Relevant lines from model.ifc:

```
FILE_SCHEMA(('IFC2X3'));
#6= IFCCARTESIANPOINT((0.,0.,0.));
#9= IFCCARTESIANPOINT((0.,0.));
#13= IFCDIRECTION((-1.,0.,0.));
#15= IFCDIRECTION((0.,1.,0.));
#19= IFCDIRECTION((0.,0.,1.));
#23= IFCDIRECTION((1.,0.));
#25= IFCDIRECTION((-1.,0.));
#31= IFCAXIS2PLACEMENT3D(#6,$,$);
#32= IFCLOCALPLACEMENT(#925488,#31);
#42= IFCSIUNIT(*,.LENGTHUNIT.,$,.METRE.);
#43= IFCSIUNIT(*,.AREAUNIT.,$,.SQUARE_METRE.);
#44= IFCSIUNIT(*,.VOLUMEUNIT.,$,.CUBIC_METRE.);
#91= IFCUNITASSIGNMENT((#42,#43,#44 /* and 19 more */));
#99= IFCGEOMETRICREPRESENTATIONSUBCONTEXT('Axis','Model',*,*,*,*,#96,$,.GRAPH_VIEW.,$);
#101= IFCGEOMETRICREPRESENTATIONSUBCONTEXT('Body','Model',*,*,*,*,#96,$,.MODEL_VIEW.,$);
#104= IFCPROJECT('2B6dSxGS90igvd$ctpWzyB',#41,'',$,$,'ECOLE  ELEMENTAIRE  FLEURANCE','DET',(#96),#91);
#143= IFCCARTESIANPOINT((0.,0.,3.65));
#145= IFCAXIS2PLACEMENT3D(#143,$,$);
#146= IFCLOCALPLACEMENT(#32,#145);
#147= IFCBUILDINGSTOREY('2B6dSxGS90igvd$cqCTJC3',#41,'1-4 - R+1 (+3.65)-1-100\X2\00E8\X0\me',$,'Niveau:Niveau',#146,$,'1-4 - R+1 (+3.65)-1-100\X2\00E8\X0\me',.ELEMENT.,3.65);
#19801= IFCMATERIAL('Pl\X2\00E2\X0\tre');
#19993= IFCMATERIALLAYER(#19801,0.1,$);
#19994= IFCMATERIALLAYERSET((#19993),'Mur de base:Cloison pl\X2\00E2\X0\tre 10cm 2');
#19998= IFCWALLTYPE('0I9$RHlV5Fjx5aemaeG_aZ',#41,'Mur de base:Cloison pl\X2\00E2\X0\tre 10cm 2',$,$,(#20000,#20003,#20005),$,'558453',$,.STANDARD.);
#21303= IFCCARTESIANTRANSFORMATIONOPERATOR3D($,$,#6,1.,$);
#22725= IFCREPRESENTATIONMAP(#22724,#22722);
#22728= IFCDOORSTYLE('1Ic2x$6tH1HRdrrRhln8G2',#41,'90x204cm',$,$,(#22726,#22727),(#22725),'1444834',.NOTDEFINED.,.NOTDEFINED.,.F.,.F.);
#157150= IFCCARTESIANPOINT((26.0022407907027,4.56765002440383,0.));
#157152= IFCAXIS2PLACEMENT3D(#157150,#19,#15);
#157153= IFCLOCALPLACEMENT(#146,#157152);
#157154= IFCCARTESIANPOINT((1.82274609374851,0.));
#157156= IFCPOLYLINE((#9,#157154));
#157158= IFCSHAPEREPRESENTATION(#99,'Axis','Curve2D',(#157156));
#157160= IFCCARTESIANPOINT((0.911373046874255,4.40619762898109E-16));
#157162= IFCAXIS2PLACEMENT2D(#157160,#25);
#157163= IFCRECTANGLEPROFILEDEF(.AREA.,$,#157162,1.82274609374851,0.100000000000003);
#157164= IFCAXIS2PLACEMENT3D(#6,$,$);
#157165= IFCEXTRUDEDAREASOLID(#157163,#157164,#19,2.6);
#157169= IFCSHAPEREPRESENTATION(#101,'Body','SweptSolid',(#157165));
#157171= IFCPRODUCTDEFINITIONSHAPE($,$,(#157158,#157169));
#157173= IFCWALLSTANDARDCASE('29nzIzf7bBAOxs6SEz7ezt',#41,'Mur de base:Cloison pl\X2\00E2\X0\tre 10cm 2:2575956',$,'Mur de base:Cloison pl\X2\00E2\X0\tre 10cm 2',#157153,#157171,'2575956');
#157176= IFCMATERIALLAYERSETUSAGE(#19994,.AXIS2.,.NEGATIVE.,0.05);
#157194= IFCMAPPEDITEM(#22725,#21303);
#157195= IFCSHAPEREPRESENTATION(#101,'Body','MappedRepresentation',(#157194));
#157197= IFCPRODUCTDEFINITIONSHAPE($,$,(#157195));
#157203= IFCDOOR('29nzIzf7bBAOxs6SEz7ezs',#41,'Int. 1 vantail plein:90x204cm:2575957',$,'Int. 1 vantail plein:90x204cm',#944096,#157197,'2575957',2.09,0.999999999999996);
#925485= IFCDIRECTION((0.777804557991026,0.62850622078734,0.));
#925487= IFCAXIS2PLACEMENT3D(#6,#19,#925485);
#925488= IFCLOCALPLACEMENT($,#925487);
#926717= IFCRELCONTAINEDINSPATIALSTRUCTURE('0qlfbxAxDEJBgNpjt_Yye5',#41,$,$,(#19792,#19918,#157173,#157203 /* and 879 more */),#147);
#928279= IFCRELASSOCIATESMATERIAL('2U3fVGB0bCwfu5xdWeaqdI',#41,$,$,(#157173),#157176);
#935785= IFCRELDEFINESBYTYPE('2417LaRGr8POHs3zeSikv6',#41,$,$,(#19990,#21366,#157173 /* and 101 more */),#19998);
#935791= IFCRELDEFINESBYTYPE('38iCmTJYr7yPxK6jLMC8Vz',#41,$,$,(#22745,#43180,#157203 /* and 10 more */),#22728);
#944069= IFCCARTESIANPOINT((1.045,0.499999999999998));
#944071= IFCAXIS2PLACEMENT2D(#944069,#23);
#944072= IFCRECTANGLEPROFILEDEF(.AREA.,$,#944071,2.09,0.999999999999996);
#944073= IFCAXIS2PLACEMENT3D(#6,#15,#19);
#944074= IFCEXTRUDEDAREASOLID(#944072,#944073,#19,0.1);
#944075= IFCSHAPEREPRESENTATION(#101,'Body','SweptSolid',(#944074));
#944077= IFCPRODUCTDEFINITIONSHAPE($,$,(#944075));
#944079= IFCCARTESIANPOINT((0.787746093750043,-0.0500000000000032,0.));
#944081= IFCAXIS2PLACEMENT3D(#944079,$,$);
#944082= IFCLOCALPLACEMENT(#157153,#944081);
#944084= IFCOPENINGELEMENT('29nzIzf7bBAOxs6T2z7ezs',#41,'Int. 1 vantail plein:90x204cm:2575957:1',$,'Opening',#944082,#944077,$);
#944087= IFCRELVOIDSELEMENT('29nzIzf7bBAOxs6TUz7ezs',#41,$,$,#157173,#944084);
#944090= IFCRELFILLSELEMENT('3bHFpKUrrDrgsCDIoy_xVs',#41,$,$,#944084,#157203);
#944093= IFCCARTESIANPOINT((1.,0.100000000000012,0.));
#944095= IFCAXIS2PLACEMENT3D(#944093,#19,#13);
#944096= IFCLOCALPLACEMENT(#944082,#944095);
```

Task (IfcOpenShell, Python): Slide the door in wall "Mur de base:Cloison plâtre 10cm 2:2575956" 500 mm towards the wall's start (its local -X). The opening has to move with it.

```python
import ifcopenshell
import ifcopenshell.api.geometry
import ifcopenshell.util.placement

model = ifcopenshell.open("model.ifc")

door = model.by_guid("29nzIzf7bBAOxs6SEz7ezs")
opening = door.FillsVoids[0].RelatingOpeningElement
wall = opening.VoidsElements[0].RelatingBuildingElement

wall_matrix = ifcopenshell.util.placement.get_local_placement(wall.ObjectPlacement)
shift = wall_matrix[:3, 0] * -0.5
before = ifcopenshell.util.placement.get_local_placement(door.ObjectPlacement)[:3, 3].copy()

# The door is placed relative to its opening, so it follows when the opening moves.
matrix = ifcopenshell.util.placement.get_local_placement(opening.ObjectPlacement)
matrix[:3, 3] += shift
ifcopenshell.api.geometry.edit_object_placement(
    model, product=opening, matrix=matrix, is_si=False, should_transform_children=True
)

after = ifcopenshell.util.placement.get_local_placement(door.ObjectPlacement)[:3, 3]
print("door moved by", (after - before).round(3) + 0.0)

model.write("model-out.ifc")
```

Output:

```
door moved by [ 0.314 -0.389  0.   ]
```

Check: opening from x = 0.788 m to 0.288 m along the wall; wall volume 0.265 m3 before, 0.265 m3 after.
